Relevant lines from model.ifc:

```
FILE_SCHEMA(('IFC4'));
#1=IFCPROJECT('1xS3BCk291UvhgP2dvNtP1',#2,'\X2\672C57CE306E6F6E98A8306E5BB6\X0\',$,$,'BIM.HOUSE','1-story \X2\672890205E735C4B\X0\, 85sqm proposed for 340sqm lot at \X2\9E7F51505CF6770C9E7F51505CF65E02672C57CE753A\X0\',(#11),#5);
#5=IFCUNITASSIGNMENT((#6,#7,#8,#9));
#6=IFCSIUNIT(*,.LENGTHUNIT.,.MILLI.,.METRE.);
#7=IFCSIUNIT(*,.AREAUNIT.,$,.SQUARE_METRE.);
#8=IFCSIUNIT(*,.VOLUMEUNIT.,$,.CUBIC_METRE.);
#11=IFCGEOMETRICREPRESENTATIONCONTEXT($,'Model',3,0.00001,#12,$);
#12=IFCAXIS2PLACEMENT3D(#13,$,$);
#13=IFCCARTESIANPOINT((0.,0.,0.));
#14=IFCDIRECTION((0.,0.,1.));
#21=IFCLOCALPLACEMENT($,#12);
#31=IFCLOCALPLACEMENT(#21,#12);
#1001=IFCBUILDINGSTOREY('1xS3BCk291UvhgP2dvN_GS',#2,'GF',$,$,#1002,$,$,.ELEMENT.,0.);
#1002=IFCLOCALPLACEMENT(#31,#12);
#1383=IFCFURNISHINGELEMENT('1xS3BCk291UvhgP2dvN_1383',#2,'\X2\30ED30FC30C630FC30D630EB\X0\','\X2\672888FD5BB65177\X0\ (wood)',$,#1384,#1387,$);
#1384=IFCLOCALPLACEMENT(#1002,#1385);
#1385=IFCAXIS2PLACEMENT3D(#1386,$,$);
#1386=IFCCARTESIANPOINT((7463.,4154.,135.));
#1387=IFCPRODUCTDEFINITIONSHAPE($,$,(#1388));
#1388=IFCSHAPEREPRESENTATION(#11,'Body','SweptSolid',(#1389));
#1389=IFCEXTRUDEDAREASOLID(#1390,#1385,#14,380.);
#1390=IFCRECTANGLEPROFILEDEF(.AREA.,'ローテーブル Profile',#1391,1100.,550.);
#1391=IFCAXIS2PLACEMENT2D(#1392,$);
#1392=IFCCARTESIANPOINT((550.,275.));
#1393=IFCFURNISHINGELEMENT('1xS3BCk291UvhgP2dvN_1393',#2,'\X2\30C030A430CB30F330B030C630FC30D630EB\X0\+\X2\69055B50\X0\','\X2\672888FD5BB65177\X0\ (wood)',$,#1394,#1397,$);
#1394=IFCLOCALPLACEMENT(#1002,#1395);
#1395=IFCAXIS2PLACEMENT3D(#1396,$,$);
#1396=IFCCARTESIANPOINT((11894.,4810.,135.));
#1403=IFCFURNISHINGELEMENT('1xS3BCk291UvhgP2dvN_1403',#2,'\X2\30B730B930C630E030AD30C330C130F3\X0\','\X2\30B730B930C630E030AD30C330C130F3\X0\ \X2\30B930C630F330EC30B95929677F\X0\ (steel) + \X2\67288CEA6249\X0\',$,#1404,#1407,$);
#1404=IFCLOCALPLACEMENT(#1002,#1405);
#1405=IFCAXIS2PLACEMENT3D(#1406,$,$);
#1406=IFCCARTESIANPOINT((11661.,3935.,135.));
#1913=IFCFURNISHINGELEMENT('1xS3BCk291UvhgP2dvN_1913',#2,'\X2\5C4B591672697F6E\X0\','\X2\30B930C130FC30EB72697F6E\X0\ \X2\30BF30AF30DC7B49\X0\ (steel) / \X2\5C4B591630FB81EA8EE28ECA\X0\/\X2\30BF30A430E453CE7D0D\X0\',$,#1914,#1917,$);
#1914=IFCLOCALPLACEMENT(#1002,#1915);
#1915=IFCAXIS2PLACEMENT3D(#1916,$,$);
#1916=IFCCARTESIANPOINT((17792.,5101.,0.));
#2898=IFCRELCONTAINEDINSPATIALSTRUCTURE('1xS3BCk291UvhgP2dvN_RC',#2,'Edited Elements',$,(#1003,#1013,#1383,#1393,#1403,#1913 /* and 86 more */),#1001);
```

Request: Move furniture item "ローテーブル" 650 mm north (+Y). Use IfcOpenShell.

```python
import ifcopenshell
import ifcopenshell.api.geometry
import ifcopenshell.util.placement
import ifcopenshell.util.unit

model = ifcopenshell.open("model.ifc")
unit_scale = ifcopenshell.util.unit.calculate_unit_scale(model)

item = model.by_id(1383)
matrix = ifcopenshell.util.placement.get_local_placement(item.ObjectPlacement)
matrix[1, 3] += 0.65 / unit_scale
ifcopenshell.api.geometry.edit_object_placement(model, product=item, matrix=matrix, is_si=False)

print(ifcopenshell.util.placement.get_local_placement(item.ObjectPlacement).round(3) + 0.0)

model.write("model_rev.ifc")
```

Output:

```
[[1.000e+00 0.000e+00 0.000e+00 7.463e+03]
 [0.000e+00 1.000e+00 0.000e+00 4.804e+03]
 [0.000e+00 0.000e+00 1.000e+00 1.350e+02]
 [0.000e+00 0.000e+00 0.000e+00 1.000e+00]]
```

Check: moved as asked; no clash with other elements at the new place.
